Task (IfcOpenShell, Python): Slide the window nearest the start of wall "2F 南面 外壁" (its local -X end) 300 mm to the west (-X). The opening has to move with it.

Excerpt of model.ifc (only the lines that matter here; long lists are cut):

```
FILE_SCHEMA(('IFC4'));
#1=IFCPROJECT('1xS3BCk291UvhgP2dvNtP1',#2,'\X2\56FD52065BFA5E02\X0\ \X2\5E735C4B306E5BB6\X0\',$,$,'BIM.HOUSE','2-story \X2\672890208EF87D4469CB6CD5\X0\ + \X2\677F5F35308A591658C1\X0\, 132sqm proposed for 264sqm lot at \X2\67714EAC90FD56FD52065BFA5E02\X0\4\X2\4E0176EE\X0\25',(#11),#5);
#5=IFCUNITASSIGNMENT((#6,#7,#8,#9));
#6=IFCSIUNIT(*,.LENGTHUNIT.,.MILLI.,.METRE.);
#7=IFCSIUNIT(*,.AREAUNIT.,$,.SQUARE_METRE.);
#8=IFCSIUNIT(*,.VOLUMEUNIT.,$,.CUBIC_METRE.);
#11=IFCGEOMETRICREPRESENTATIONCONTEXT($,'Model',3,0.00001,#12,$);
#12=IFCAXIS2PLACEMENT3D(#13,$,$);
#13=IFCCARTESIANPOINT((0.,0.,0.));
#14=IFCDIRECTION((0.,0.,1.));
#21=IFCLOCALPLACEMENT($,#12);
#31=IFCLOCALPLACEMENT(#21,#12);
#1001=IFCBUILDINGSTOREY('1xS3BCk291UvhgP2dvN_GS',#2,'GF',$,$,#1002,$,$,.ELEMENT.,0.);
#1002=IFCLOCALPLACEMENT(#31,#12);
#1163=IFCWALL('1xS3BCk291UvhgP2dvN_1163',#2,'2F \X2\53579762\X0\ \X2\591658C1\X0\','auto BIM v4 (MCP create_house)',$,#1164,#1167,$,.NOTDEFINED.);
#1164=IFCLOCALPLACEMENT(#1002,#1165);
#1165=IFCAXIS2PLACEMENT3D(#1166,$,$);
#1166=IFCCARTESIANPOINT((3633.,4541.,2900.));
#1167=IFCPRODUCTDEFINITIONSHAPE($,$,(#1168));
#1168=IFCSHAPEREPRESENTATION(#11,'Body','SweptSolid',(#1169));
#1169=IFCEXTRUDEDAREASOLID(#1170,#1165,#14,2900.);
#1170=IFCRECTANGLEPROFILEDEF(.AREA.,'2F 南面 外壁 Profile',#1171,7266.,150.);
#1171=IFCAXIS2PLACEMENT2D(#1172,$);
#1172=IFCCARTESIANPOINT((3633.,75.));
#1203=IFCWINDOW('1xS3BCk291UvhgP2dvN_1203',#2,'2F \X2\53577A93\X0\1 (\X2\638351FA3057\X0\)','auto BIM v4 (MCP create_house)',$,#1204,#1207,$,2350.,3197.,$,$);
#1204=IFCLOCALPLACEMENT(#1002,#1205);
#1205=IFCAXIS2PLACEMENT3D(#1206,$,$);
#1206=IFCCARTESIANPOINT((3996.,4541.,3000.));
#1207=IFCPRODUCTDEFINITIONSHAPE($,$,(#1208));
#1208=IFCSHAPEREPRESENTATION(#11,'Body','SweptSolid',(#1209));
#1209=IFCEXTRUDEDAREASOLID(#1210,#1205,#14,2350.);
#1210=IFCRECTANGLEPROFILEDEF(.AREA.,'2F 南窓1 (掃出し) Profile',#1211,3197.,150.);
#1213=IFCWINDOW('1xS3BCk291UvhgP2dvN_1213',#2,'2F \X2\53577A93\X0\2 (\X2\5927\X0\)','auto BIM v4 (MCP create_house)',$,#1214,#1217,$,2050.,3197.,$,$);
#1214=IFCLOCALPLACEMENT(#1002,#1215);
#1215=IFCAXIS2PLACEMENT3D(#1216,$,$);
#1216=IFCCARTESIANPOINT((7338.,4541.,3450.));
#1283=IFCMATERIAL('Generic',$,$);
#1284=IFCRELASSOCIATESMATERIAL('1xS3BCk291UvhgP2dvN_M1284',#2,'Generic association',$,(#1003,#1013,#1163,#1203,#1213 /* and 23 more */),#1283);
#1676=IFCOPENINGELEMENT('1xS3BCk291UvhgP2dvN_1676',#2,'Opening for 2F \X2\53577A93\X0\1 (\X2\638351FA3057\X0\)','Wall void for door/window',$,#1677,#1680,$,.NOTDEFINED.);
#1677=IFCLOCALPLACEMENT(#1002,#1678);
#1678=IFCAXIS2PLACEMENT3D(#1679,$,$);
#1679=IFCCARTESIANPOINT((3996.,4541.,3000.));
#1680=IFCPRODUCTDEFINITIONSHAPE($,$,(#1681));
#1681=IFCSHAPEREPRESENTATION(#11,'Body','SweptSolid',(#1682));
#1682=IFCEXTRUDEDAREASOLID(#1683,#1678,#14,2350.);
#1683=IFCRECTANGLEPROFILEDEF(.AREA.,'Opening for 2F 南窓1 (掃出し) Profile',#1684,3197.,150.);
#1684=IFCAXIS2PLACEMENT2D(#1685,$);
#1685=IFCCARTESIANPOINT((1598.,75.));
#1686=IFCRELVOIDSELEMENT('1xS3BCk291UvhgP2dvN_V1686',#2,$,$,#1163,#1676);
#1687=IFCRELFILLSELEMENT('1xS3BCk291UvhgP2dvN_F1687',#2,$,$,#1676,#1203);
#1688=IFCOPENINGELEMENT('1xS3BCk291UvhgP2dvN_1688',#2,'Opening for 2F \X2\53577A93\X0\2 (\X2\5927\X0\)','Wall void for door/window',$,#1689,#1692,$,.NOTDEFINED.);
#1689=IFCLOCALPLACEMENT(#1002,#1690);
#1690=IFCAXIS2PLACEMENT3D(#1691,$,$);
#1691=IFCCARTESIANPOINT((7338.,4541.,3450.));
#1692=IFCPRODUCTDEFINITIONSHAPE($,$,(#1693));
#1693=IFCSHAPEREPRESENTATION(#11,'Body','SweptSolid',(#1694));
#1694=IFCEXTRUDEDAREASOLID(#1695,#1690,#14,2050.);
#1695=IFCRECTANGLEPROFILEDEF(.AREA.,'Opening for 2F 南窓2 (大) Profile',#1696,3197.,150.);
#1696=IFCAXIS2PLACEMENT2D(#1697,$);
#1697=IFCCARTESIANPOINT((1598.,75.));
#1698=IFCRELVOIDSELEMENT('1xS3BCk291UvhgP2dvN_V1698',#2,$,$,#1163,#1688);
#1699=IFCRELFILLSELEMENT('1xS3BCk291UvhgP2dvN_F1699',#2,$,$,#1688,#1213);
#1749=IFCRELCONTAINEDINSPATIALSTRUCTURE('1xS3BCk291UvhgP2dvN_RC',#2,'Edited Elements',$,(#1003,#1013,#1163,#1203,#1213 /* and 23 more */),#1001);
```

```python
import ifcopenshell
import ifcopenshell.api.geometry
import ifcopenshell.util.placement

model = ifcopenshell.open("model.ifc")

window = model.by_guid("1xS3BCk291UvhgP2dvN_1203")
opening = window.FillsVoids[0].RelatingOpeningElement
wall = opening.VoidsElements[0].RelatingBuildingElement

wall_matrix = ifcopenshell.util.placement.get_local_placement(wall.ObjectPlacement)
shift = wall_matrix[:3, 0] * -300.0
before = ifcopenshell.util.placement.get_local_placement(window.ObjectPlacement)[:3, 3].copy()

# The window is not placed relative to its opening, so move both.
for product in (opening, window):
    matrix = ifcopenshell.util.placement.get_local_placement(product.ObjectPlacement)
    matrix[:3, 3] += shift
    ifcopenshell.api.geometry.edit_object_placement(model, product=product, matrix=matrix, is_si=False)

after = ifcopenshell.util.placement.get_local_placement(window.ObjectPlacement)[:3, 3]
print("window moved by", (after - before).round(3) + 0.0)

model.write("model-out.ifc")
```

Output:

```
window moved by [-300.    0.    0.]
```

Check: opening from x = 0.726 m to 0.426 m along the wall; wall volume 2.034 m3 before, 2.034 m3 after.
